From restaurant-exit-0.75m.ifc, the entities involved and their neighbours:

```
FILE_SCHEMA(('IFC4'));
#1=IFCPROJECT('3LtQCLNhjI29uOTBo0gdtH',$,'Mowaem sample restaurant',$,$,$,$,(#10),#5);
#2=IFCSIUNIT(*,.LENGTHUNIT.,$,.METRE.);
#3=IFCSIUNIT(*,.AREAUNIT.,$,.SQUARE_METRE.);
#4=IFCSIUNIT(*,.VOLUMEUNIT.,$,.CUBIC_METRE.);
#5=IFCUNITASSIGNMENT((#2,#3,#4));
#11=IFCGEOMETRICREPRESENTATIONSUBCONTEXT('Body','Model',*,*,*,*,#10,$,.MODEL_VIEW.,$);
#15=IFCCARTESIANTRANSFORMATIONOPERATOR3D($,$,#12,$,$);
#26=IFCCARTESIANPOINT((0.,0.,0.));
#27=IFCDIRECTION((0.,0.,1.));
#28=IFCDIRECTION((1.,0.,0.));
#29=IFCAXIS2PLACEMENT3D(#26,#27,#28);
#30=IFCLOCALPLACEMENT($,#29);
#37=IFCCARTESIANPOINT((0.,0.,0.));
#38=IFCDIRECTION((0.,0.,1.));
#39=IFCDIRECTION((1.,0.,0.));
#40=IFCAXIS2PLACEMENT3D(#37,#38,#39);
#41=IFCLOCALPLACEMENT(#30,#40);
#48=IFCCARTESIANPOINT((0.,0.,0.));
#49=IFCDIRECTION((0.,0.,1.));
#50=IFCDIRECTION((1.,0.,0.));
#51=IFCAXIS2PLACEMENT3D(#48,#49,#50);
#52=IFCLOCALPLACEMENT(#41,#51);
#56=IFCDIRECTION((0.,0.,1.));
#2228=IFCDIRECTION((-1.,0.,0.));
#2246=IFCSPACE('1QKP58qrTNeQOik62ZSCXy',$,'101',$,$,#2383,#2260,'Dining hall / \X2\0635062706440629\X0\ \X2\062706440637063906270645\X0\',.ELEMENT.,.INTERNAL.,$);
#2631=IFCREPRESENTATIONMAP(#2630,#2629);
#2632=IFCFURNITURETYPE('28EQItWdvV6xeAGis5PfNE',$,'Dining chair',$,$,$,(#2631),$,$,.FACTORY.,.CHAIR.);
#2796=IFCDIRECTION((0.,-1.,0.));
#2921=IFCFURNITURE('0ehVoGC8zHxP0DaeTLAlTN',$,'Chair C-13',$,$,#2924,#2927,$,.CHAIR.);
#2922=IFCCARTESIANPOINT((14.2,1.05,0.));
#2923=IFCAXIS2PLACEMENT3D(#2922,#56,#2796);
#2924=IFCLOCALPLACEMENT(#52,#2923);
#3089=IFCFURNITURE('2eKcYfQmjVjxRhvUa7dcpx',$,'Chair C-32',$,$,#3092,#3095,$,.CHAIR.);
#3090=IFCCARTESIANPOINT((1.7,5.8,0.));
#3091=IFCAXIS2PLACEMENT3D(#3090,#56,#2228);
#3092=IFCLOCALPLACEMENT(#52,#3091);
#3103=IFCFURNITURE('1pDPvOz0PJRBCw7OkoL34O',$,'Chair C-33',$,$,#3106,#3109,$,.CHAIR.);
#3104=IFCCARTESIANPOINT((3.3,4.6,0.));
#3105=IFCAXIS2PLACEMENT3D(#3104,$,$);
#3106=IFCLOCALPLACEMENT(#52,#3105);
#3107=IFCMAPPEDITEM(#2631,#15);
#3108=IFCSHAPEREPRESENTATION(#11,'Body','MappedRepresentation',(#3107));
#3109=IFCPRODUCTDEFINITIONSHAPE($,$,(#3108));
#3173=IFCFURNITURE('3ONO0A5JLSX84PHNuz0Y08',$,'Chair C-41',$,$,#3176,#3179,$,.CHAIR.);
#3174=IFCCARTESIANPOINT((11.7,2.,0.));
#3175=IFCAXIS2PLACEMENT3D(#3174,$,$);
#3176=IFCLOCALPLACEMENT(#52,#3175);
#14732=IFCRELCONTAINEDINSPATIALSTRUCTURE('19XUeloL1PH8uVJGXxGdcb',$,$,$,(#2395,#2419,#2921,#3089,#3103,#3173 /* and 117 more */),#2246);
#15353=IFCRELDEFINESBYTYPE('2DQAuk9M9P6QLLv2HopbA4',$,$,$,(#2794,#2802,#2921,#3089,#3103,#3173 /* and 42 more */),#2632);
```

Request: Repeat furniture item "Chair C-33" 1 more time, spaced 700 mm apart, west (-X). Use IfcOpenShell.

```python
import numpy as np
import ifcopenshell
import ifcopenshell.api.geometry
import ifcopenshell.api.root
import ifcopenshell.util.element
import ifcopenshell.util.placement

model = ifcopenshell.open("restaurant-exit-0.75m.ifc")

source = model.by_guid("1pDPvOz0PJRBCw7OkoL34O")
base = ifcopenshell.util.placement.get_local_placement(source.ObjectPlacement)
step = np.array([-1.0, 0.0, 0.0]) * 0.7

for i in range(1, 2):
    copy = ifcopenshell.api.root.copy_class(model, product=source)
    copy.Representation = ifcopenshell.util.element.copy_deep(
        model, source.Representation, exclude=["IfcGeometricRepresentationContext", "IfcRepresentationMap"]
    )
    matrix = base.copy()
    matrix[:3, 3] += i * step
    print("added at", matrix[:3, 3].round(3) + 0.0)
    ifcopenshell.api.geometry.edit_object_placement(model, product=copy, matrix=matrix, is_si=False)

model.write("restaurant-exit-0.75m-out.ifc")
```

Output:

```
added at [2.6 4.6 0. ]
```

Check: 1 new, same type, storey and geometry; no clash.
